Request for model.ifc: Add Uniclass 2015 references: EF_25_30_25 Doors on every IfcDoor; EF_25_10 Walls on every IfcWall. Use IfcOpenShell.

First a look at what the model holds.

```python
import ifcopenshell

model = ifcopenshell.open("model.ifc")
print(model.schema)
print("classifications:", [c.Name for c in model.by_type("IfcClassification")])
for ifc_class in ("IfcDoor", "IfcRoof", "IfcStair", "IfcWall", "IfcWindow"):
    print(ifc_class, len(model.by_type(ifc_class)))
```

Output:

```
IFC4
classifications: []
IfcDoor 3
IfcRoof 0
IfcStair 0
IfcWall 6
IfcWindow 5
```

```python
import ifcopenshell
import ifcopenshell.api.classification

model = ifcopenshell.open("model.ifc")

system = ifcopenshell.api.classification.add_classification(model, classification="Uniclass 2015")

codes = {
    "IfcDoor": ("EF_25_30_25", "Doors"),
    "IfcWall": ("EF_25_10", "Walls"),
}
for ifc_class, (code, name) in codes.items():
    products = model.by_type(ifc_class)
    ifcopenshell.api.classification.add_reference(
        model, products=products, classification=system, identification=code, name=name
    )
    print(code, len(products))

model.write("model_updated.ifc")
```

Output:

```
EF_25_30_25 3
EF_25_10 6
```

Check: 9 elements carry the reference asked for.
